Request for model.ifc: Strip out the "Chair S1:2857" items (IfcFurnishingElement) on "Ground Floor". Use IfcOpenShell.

First a look at what the model holds.

```python
import ifcopenshell
import ifcopenshell.util.element

model = ifcopenshell.open("model.ifc")
print(model.schema)
storey = next(s for s in model.by_type("IfcBuildingStorey") if s.Name == "Ground Floor")
furniture = [e for e in ifcopenshell.util.element.get_decomposition(storey) if e.is_a("IfcFurnishingElement")]
seen = {}
for e in furniture:
    element_type = ifcopenshell.util.element.get_type(e)
    name = element_type.Name if element_type not in (None, e) else None
    seen[name] = seen.get(name, 0) + 1
for name, count in sorted(seen.items(), key=str):
    print(count, "x", name)
```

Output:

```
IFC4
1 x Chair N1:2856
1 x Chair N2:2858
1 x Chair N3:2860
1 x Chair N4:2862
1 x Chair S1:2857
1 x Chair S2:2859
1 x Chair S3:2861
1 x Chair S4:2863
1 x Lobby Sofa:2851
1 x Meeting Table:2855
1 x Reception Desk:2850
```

```python
import ifcopenshell
import ifcopenshell.api.root
import ifcopenshell.util.element

model = ifcopenshell.open("model.ifc")

storey = next(s for s in model.by_type("IfcBuildingStorey") if s.Name == "Ground Floor")
furniture = [e for e in ifcopenshell.util.element.get_decomposition(storey) if e.is_a("IfcFurnishingElement")]
targets = [e for e in furniture if (t := ifcopenshell.util.element.get_type(e)) not in (None, e) and t.Name == "Chair S1:2857"]

for e in targets:
    ifcopenshell.api.root.remove_product(model, product=e)
print(len(targets), "removed")

model.write("model_rev.ifc")
```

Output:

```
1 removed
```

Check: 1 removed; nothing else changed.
